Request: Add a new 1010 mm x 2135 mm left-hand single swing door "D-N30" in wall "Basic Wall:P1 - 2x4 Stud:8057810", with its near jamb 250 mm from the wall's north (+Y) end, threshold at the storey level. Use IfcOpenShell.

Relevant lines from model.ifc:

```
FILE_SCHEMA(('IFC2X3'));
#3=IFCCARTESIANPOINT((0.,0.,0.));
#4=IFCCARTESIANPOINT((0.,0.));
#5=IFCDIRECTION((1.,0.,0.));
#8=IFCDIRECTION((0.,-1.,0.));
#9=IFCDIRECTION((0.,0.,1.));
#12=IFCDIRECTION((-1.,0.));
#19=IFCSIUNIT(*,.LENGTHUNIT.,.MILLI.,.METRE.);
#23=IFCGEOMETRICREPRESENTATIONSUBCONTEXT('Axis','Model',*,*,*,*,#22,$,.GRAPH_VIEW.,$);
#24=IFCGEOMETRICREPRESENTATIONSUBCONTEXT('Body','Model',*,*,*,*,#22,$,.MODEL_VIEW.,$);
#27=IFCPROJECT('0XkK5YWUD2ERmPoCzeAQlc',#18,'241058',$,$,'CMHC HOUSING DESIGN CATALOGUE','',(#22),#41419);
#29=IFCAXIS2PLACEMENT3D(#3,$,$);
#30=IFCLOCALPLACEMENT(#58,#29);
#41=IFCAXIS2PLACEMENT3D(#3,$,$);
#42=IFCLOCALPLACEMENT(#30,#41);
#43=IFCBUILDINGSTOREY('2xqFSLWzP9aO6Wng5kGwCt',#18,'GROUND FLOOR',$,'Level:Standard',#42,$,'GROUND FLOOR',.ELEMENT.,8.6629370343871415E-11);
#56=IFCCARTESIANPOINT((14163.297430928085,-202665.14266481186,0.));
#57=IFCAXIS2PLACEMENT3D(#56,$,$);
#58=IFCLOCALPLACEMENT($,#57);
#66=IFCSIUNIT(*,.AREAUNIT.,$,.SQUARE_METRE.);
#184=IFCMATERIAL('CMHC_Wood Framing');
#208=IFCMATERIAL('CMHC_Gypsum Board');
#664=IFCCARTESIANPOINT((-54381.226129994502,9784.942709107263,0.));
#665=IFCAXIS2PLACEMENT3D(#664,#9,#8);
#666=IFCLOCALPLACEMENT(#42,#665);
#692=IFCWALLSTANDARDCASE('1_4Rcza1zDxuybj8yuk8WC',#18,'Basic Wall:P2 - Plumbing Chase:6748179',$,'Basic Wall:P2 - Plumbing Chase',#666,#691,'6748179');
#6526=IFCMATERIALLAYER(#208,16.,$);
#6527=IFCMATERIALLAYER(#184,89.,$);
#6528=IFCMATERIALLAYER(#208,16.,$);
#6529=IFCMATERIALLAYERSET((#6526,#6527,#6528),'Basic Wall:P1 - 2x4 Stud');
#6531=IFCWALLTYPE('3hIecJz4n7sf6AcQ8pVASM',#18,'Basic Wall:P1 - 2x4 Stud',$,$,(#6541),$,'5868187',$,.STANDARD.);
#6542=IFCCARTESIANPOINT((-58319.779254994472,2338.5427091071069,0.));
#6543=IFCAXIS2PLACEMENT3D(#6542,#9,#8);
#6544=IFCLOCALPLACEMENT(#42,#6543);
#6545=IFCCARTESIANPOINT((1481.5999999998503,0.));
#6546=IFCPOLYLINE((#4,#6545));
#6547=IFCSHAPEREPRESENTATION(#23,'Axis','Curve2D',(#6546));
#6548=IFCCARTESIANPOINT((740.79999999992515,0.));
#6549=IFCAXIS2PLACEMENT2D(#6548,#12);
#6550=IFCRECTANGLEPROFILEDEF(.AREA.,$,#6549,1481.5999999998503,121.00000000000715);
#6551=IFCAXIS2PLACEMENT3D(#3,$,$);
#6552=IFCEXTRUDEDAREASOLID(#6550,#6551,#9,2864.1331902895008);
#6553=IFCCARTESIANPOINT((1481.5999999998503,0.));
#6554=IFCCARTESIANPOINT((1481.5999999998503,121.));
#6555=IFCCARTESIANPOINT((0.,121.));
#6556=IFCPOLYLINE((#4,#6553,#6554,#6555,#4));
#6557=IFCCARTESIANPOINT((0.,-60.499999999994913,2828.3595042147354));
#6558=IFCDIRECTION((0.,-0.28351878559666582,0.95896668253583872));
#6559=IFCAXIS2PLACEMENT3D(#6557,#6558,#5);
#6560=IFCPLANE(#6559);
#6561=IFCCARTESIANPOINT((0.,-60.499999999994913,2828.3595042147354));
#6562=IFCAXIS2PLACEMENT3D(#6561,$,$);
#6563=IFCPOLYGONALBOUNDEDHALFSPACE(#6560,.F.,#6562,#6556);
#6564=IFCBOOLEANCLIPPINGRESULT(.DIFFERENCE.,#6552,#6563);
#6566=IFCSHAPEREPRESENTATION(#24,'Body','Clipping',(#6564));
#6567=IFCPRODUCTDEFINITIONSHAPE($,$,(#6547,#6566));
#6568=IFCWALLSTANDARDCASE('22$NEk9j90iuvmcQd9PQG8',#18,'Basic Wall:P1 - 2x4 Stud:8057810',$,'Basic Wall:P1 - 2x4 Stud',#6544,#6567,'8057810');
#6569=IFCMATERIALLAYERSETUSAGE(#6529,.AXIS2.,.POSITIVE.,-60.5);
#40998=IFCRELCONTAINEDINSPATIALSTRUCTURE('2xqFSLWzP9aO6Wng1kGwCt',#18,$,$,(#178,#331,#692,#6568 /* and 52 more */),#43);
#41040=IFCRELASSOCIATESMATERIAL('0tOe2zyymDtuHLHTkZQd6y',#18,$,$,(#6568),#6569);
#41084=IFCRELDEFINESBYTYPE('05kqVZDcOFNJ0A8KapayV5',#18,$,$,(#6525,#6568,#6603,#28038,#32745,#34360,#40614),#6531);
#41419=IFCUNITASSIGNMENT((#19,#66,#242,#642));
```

```python
import numpy as np
import ifcopenshell
import ifcopenshell.api.feature
import ifcopenshell.api.geometry
import ifcopenshell.api.root
import ifcopenshell.api.spatial
import ifcopenshell.api.type
import ifcopenshell.geom
import ifcopenshell.util.element
import ifcopenshell.util.placement
import ifcopenshell.util.representation
import ifcopenshell.util.shape
import ifcopenshell.util.unit

model = ifcopenshell.open("model.ifc")
unit_scale = ifcopenshell.util.unit.calculate_unit_scale(model)
settings = ifcopenshell.geom.settings()


def volume(element):
    """Net volume in cubic metres, openings subtracted."""
    shape = ifcopenshell.geom.create_shape(settings, element)
    return ifcopenshell.util.shape.get_volume(shape.geometry)


wall = model.by_guid("22$NEk9j90iuvmcQd9PQG8")
storey = ifcopenshell.util.element.get_container(wall, ifc_class="IfcBuildingStorey")
context = ifcopenshell.util.representation.get_context(model, "Model", "Body", "MODEL_VIEW")
before = volume(wall)

width, height, from_end, sill = 1.01, 2.135, 0.25, 0.0  # metres

# The wall runs along its own X axis, and the end named is its -X end.
wall_shape = ifcopenshell.geom.create_shape(settings, wall)
x, y, z = ifcopenshell.util.shape.get_vertices(wall_shape.geometry).T
start = x.min() + from_end
face, thickness = float(y.min()), float(y.max() - y.min())
wall_matrix = ifcopenshell.util.placement.get_local_placement(wall.ObjectPlacement)
level = ifcopenshell.util.placement.get_local_placement(storey.ObjectPlacement)[2, 3]


def in_wall(x, y):
    """Placement at x, y metres in the wall's axes, at sill height."""
    matrix = wall_matrix.copy()
    matrix[:, 3] = wall_matrix @ np.array([x / unit_scale, y / unit_scale, 0.0, 1.0])
    matrix[2, 3] = level + sill / unit_scale
    return matrix


# Opening: a box that overshoots both wall faces by 50 mm.
opening = ifcopenshell.api.root.create_entity(model, ifc_class="IfcOpeningElement")
box = ifcopenshell.api.geometry.add_wall_representation(
    model, context=context, length=width, height=height, thickness=thickness + 0.1
)
ifcopenshell.api.geometry.assign_representation(model, product=opening, representation=box)
ifcopenshell.api.geometry.edit_object_placement(model, product=opening, matrix=in_wall(start, face - 0.05), is_si=False)
ifcopenshell.api.feature.add_feature(model, feature=opening, element=wall)

door = ifcopenshell.api.root.create_entity(model, ifc_class="IfcDoor", name="D-N30")
door.OverallWidth, door.OverallHeight = width / unit_scale, height / unit_scale
body = ifcopenshell.api.geometry.add_door_representation(
    model,
    context=context,
    overall_width=door.OverallWidth,
    overall_height=door.OverallHeight,
    operation_type="SINGLE_SWING_LEFT",
    lining_properties={"LiningDepth": thickness / unit_scale, "ThresholdDepth": thickness / unit_scale},
)
ifcopenshell.api.geometry.assign_representation(model, product=door, representation=body)
ifcopenshell.api.spatial.assign_container(model, products=[door], relating_structure=storey)
fills = ifcopenshell.api.feature.add_filling(model, opening=opening, element=door)
fills.OwnerHistory = door.OwnerHistory  # required in IFC2X3

# IFC2X3 keeps the operation on the door style.
style = ifcopenshell.api.root.create_entity(model, ifc_class="IfcDoorStyle", name="D-N30")
style.OperationType, style.ConstructionType = "SINGLE_SWING_LEFT", "NOTDEFINED"
style.ParameterTakesPrecedence = style.Sizeable = False
ifcopenshell.api.type.assign_type(model, related_objects=[door], relating_type=style)

# The lining spans the wall, so the door starts at the wall face.
ifcopenshell.api.geometry.edit_object_placement(model, product=door, matrix=in_wall(start, face), is_si=False)

after = volume(wall)

print(f"wall volume {before:.3f} -> {after:.3f} m3")

model.write("model-out.ifc")
```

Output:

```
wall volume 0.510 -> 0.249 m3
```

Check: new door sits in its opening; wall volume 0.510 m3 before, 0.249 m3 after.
